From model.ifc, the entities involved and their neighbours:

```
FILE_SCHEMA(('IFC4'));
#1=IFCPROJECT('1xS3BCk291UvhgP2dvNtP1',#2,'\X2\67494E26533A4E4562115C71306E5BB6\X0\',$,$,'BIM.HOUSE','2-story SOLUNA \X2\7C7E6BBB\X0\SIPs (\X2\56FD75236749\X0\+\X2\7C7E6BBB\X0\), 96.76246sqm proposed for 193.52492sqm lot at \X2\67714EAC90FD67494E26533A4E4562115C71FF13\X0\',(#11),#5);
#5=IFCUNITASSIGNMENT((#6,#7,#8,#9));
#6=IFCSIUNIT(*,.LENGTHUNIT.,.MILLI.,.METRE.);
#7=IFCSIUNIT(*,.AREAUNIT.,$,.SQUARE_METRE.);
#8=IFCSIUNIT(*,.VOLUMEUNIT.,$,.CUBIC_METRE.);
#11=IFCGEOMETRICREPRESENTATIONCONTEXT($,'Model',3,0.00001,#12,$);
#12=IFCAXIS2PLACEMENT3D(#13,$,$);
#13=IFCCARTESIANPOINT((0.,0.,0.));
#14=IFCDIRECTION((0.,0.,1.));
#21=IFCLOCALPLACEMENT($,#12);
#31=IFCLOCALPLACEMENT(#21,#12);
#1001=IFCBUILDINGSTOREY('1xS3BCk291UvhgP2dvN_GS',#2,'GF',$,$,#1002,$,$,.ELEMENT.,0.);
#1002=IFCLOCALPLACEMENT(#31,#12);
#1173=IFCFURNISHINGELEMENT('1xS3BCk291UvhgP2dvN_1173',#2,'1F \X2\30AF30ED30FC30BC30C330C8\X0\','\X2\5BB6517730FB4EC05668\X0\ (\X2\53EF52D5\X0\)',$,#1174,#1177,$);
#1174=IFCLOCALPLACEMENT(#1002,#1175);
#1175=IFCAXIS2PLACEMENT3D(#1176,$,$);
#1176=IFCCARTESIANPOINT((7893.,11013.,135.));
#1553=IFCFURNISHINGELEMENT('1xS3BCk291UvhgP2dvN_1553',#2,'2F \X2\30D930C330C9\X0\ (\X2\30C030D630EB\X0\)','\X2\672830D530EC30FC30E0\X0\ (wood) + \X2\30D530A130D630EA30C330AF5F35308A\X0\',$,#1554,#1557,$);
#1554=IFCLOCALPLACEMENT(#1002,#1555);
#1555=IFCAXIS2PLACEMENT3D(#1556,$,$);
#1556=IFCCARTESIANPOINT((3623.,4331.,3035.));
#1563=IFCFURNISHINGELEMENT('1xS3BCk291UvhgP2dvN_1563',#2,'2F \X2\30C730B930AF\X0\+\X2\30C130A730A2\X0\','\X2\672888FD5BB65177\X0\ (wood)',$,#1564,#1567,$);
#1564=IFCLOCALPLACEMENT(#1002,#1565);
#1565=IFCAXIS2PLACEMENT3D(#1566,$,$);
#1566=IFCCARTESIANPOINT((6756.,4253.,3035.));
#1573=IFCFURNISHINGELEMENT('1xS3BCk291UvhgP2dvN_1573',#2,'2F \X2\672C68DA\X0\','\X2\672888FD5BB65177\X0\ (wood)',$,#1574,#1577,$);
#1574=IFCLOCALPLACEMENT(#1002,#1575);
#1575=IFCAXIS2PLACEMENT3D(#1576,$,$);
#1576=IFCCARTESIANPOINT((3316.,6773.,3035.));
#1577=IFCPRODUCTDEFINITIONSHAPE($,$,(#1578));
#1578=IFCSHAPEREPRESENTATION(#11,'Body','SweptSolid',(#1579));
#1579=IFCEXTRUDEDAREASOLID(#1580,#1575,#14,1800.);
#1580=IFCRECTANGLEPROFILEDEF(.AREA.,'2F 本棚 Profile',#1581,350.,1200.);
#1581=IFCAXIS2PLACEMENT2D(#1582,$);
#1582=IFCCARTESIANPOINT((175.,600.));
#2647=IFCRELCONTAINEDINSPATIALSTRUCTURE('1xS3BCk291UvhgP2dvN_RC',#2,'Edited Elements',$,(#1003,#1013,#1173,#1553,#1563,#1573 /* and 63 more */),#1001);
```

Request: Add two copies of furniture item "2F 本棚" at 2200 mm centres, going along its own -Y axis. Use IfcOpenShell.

```python
import ifcopenshell
import ifcopenshell.api.geometry
import ifcopenshell.api.root
import ifcopenshell.util.element
import ifcopenshell.util.placement

model = ifcopenshell.open("model.ifc")


def reuse_history(source, copy):
    """copy_class also copies each property set's owner history, people and application; keep the originals."""
    for rel in copy.IsDefinedBy:
        if rel.is_a("IfcRelDefinesByProperties") and (history := rel.RelatingPropertyDefinition.OwnerHistory):
            rel.RelatingPropertyDefinition.OwnerHistory = source.OwnerHistory
            ifcopenshell.util.element.remove_deep2(model, history)


source = model.by_guid("1xS3BCk291UvhgP2dvN_1573")
base = ifcopenshell.util.placement.get_local_placement(source.ObjectPlacement)
step = -base[:3, 1] * 2200.0

for i in range(1, 3):
    copy = ifcopenshell.api.root.copy_class(model, product=source)
    copy.Representation = ifcopenshell.util.element.copy_deep(
        model, source.Representation, exclude=["IfcGeometricRepresentationContext", "IfcRepresentationMap"]
    )
    reuse_history(source, copy)
    matrix = base.copy()
    matrix[:3, 3] += i * step
    print("added at", matrix[:3, 3].round(3) + 0.0)
    ifcopenshell.api.geometry.edit_object_placement(model, product=copy, matrix=matrix, is_si=False)

model.write("model-out.ifc")
```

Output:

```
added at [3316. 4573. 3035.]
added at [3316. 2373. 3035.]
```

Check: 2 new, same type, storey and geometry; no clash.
